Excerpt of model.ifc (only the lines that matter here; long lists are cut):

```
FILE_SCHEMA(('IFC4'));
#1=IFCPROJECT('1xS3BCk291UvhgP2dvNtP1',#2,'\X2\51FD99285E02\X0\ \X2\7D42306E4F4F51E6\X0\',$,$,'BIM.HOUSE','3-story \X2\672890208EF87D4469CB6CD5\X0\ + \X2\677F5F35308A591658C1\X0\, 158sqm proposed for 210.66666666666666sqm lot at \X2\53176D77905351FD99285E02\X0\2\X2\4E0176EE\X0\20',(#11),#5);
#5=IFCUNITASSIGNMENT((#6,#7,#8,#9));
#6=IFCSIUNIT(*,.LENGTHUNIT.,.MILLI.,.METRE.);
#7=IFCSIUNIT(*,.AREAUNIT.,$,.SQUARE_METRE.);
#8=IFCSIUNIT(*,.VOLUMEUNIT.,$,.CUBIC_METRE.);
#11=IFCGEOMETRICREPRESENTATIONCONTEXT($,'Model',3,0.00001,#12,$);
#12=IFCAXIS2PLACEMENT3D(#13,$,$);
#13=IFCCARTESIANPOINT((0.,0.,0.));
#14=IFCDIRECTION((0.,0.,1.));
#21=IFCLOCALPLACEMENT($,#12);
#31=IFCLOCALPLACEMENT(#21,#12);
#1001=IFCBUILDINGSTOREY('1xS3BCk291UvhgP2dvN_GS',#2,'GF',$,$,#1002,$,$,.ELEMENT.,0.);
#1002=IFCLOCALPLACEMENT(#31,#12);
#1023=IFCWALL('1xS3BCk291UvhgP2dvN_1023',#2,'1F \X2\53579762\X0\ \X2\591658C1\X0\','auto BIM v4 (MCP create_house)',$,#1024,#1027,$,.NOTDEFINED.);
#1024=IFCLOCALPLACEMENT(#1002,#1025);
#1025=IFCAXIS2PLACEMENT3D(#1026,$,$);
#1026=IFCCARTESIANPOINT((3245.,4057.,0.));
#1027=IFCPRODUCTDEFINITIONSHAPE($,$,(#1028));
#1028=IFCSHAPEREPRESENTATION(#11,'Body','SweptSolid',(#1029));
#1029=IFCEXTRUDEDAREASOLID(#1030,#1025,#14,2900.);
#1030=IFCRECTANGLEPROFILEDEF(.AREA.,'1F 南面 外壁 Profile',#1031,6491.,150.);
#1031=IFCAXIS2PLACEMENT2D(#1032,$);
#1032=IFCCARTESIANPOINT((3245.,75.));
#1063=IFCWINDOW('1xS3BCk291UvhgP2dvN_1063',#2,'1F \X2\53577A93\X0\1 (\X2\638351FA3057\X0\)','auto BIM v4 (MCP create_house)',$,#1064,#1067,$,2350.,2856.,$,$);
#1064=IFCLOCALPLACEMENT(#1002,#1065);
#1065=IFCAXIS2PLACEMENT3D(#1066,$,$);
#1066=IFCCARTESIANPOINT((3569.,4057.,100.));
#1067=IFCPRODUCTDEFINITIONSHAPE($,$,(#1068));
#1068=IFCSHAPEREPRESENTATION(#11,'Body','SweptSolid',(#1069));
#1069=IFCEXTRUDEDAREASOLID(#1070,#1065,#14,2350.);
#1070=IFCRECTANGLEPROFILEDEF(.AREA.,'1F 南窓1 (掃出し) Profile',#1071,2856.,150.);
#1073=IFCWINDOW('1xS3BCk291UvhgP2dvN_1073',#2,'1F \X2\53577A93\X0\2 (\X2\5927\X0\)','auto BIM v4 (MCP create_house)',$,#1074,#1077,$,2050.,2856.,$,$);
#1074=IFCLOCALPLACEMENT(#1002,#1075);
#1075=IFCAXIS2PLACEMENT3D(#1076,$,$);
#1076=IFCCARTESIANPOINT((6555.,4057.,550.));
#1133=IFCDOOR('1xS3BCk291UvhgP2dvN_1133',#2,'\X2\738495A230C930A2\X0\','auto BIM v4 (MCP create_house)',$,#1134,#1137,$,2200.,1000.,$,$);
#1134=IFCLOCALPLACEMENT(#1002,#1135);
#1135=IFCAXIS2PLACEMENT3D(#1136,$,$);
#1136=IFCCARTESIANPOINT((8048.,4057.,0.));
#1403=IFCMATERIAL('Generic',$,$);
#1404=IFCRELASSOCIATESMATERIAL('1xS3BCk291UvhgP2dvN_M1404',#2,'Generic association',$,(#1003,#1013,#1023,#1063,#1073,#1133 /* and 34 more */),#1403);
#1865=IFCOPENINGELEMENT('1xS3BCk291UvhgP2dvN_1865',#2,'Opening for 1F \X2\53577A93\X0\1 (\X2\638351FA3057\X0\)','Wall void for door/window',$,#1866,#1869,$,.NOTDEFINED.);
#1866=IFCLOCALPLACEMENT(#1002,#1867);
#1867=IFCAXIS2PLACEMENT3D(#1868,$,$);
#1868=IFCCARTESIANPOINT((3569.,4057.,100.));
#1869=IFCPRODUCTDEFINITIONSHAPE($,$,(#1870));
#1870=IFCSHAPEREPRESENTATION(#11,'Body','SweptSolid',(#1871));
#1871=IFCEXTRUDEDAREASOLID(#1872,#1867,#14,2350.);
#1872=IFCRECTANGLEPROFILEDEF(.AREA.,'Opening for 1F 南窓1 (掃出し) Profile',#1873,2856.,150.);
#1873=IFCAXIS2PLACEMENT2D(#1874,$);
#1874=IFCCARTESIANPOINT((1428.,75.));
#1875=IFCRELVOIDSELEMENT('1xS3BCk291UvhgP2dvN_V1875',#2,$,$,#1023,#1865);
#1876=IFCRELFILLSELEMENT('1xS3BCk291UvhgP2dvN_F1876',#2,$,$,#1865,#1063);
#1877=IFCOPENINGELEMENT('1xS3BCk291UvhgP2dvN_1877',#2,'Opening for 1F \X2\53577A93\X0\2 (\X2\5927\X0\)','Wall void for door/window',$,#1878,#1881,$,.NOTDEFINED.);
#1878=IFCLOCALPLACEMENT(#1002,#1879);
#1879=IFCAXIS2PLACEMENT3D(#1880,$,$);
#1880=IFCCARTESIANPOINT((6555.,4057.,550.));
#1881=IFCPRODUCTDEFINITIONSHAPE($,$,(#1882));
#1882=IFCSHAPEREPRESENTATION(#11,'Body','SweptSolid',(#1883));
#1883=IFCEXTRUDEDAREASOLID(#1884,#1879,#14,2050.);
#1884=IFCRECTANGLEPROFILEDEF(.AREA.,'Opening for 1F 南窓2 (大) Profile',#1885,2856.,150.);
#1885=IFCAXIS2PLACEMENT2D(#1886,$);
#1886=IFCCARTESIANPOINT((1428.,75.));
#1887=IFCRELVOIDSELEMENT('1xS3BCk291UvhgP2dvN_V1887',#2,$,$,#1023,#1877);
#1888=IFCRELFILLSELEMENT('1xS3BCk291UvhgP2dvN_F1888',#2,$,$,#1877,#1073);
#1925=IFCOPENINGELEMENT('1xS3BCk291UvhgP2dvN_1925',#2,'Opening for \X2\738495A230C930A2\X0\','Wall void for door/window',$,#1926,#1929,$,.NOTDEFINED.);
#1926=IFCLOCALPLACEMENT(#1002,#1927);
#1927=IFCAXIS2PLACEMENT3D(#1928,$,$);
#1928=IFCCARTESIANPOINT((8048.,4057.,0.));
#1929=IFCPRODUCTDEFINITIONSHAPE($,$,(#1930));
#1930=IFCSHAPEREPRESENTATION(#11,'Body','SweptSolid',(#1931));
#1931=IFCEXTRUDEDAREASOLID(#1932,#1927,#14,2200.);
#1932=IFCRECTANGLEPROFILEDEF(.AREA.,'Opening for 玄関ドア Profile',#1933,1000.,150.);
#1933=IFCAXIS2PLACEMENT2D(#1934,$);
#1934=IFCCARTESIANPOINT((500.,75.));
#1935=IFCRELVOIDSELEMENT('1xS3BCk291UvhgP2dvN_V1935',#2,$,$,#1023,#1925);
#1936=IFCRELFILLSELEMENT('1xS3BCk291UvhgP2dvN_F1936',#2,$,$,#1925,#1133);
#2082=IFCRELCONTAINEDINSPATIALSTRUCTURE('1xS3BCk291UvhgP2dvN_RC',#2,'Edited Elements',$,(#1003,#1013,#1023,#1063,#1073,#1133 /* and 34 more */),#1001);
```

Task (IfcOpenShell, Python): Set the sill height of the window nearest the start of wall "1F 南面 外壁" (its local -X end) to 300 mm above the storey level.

```python
import numpy as np
import ifcopenshell
import ifcopenshell.api.geometry
import ifcopenshell.geom
import ifcopenshell.util.element
import ifcopenshell.util.placement
import ifcopenshell.util.shape
import ifcopenshell.util.unit

model = ifcopenshell.open("model.ifc")
unit_scale = ifcopenshell.util.unit.calculate_unit_scale(model)

window = model.by_guid("1xS3BCk291UvhgP2dvN_1063")
opening = window.FillsVoids[0].RelatingOpeningElement
storey = ifcopenshell.util.element.get_container(window, ifc_class="IfcBuildingStorey")
level = ifcopenshell.util.placement.get_local_placement(storey.ObjectPlacement)[2, 3]

# The opening's origin need not be at the sill, so measure its lowest point.
shape = ifcopenshell.geom.create_shape(ifcopenshell.geom.settings(), opening)
bottom = ifcopenshell.util.shape.get_shape_bottom_elevation(shape, shape.geometry) / unit_scale
dz = level + 0.3 / unit_scale - bottom

shift = np.array([0.0, 0.0, dz])
# The window is not placed relative to its opening, so move both.
for product in (opening, window):
    matrix = ifcopenshell.util.placement.get_local_placement(product.ObjectPlacement)
    matrix[:3, 3] += shift
    ifcopenshell.api.geometry.edit_object_placement(model, product=product, matrix=matrix, is_si=False)

print(f"moved by {dz * unit_scale:+.3f} m")

model.write("model_rev.ifc")
```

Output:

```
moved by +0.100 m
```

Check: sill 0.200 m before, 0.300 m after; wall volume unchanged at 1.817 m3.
